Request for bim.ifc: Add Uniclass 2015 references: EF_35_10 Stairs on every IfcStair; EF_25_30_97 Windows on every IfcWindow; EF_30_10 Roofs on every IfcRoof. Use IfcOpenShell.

First a look at what the model holds.

```python
import ifcopenshell

model = ifcopenshell.open("bim.ifc")
print(model.schema)
print("classifications:", [c.Name for c in model.by_type("IfcClassification")])
for ifc_class in ("IfcDoor", "IfcRoof", "IfcStair", "IfcWall", "IfcWindow"):
    print(ifc_class, len(model.by_type(ifc_class)))
```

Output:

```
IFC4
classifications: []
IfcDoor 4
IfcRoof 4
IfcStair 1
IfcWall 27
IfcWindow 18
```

```python
import ifcopenshell
import ifcopenshell.api.classification

model = ifcopenshell.open("bim.ifc")

system = ifcopenshell.api.classification.add_classification(model, classification="Uniclass 2015")

codes = {
    "IfcStair": ("EF_35_10", "Stairs"),
    "IfcWindow": ("EF_25_30_97", "Windows"),
    "IfcRoof": ("EF_30_10", "Roofs"),
}
for ifc_class, (code, name) in codes.items():
    products = model.by_type(ifc_class)
    ifcopenshell.api.classification.add_reference(
        model, products=products, classification=system, identification=code, name=name
    )
    print(code, len(products))

model.write("bim_rev.ifc")
```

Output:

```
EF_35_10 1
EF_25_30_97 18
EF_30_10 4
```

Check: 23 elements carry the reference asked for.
